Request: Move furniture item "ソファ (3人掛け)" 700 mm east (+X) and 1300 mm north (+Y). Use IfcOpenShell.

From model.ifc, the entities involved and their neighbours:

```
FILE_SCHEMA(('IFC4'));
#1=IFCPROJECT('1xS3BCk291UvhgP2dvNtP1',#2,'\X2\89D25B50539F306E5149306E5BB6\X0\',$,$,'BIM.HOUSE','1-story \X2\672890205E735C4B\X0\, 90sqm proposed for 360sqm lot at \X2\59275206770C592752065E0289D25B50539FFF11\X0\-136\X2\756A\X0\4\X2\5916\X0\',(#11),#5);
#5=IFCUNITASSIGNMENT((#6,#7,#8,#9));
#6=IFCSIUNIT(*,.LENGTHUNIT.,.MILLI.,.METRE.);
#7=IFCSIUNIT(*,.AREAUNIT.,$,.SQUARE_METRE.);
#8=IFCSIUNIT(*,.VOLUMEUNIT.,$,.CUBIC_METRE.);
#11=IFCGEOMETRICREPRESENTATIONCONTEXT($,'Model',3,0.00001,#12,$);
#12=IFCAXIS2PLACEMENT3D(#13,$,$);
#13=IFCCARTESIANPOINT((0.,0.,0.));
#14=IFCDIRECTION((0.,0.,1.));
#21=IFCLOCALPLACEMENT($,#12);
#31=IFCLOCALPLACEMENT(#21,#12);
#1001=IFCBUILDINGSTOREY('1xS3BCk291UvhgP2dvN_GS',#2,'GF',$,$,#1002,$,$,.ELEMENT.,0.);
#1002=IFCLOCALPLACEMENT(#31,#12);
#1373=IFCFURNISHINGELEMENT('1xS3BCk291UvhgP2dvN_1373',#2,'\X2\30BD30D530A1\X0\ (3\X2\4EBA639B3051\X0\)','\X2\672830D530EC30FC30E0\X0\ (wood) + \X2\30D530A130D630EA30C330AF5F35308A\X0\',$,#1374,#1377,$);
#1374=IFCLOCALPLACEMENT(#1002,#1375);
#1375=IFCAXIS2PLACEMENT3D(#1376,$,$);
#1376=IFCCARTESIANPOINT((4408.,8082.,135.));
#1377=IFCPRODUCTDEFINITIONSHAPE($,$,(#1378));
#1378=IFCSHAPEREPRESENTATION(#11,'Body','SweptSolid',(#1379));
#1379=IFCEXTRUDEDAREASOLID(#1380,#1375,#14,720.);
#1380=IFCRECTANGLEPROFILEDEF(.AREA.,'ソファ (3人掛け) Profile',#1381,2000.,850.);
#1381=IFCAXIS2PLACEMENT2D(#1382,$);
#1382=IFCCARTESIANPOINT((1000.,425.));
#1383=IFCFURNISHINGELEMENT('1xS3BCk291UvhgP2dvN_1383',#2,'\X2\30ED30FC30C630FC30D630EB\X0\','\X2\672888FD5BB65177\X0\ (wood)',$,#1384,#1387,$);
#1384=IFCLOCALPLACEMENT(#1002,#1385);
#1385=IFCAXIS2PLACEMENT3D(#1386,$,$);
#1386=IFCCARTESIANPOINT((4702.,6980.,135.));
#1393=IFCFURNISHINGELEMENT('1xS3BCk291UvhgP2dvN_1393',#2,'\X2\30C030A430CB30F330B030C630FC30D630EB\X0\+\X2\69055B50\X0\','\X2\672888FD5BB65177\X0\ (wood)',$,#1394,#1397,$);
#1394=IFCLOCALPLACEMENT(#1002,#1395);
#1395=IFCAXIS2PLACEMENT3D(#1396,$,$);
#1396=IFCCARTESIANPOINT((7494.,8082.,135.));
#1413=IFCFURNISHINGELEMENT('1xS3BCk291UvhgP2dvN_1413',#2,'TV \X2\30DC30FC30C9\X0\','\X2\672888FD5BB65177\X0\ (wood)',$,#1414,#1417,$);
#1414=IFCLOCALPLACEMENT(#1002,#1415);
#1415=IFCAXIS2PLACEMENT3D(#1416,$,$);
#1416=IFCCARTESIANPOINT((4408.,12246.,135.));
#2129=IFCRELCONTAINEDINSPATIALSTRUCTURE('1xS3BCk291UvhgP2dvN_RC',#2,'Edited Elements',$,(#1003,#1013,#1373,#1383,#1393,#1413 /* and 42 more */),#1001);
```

```python
import ifcopenshell
import ifcopenshell.api.geometry
import ifcopenshell.util.placement
import ifcopenshell.util.unit

model = ifcopenshell.open("model.ifc")
unit_scale = ifcopenshell.util.unit.calculate_unit_scale(model)

item = model.by_id(1373)
matrix = ifcopenshell.util.placement.get_local_placement(item.ObjectPlacement)
matrix[0, 3] += 0.7 / unit_scale
matrix[1, 3] += 1.3 / unit_scale
ifcopenshell.api.geometry.edit_object_placement(model, product=item, matrix=matrix, is_si=False)

print(ifcopenshell.util.placement.get_local_placement(item.ObjectPlacement).round(3) + 0.0)

model.write("model_v2.ifc")
```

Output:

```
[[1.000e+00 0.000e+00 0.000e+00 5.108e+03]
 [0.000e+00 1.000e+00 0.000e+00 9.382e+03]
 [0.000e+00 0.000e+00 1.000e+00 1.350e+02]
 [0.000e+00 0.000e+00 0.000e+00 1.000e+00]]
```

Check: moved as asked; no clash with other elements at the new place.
